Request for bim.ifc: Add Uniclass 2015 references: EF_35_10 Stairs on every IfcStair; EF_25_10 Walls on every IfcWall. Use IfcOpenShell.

First a look at what the model holds.

```python
import ifcopenshell

model = ifcopenshell.open("bim.ifc")
print(model.schema)
print("classifications:", [c.Name for c in model.by_type("IfcClassification")])
for ifc_class in ("IfcDoor", "IfcRoof", "IfcStair", "IfcWall", "IfcWindow"):
    print(ifc_class, len(model.by_type(ifc_class)))
```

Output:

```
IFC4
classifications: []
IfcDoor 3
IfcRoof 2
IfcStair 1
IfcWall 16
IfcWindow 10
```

```python
import ifcopenshell
import ifcopenshell.api.classification

model = ifcopenshell.open("bim.ifc")

system = ifcopenshell.api.classification.add_classification(model, classification="Uniclass 2015")

codes = {
    "IfcStair": ("EF_35_10", "Stairs"),
    "IfcWall": ("EF_25_10", "Walls"),
}
for ifc_class, (code, name) in codes.items():
    products = model.by_type(ifc_class)
    ifcopenshell.api.classification.add_reference(
        model, products=products, classification=system, identification=code, name=name
    )
    print(code, len(products))

model.write("bim_rev.ifc")
```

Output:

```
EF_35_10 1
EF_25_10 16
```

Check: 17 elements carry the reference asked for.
